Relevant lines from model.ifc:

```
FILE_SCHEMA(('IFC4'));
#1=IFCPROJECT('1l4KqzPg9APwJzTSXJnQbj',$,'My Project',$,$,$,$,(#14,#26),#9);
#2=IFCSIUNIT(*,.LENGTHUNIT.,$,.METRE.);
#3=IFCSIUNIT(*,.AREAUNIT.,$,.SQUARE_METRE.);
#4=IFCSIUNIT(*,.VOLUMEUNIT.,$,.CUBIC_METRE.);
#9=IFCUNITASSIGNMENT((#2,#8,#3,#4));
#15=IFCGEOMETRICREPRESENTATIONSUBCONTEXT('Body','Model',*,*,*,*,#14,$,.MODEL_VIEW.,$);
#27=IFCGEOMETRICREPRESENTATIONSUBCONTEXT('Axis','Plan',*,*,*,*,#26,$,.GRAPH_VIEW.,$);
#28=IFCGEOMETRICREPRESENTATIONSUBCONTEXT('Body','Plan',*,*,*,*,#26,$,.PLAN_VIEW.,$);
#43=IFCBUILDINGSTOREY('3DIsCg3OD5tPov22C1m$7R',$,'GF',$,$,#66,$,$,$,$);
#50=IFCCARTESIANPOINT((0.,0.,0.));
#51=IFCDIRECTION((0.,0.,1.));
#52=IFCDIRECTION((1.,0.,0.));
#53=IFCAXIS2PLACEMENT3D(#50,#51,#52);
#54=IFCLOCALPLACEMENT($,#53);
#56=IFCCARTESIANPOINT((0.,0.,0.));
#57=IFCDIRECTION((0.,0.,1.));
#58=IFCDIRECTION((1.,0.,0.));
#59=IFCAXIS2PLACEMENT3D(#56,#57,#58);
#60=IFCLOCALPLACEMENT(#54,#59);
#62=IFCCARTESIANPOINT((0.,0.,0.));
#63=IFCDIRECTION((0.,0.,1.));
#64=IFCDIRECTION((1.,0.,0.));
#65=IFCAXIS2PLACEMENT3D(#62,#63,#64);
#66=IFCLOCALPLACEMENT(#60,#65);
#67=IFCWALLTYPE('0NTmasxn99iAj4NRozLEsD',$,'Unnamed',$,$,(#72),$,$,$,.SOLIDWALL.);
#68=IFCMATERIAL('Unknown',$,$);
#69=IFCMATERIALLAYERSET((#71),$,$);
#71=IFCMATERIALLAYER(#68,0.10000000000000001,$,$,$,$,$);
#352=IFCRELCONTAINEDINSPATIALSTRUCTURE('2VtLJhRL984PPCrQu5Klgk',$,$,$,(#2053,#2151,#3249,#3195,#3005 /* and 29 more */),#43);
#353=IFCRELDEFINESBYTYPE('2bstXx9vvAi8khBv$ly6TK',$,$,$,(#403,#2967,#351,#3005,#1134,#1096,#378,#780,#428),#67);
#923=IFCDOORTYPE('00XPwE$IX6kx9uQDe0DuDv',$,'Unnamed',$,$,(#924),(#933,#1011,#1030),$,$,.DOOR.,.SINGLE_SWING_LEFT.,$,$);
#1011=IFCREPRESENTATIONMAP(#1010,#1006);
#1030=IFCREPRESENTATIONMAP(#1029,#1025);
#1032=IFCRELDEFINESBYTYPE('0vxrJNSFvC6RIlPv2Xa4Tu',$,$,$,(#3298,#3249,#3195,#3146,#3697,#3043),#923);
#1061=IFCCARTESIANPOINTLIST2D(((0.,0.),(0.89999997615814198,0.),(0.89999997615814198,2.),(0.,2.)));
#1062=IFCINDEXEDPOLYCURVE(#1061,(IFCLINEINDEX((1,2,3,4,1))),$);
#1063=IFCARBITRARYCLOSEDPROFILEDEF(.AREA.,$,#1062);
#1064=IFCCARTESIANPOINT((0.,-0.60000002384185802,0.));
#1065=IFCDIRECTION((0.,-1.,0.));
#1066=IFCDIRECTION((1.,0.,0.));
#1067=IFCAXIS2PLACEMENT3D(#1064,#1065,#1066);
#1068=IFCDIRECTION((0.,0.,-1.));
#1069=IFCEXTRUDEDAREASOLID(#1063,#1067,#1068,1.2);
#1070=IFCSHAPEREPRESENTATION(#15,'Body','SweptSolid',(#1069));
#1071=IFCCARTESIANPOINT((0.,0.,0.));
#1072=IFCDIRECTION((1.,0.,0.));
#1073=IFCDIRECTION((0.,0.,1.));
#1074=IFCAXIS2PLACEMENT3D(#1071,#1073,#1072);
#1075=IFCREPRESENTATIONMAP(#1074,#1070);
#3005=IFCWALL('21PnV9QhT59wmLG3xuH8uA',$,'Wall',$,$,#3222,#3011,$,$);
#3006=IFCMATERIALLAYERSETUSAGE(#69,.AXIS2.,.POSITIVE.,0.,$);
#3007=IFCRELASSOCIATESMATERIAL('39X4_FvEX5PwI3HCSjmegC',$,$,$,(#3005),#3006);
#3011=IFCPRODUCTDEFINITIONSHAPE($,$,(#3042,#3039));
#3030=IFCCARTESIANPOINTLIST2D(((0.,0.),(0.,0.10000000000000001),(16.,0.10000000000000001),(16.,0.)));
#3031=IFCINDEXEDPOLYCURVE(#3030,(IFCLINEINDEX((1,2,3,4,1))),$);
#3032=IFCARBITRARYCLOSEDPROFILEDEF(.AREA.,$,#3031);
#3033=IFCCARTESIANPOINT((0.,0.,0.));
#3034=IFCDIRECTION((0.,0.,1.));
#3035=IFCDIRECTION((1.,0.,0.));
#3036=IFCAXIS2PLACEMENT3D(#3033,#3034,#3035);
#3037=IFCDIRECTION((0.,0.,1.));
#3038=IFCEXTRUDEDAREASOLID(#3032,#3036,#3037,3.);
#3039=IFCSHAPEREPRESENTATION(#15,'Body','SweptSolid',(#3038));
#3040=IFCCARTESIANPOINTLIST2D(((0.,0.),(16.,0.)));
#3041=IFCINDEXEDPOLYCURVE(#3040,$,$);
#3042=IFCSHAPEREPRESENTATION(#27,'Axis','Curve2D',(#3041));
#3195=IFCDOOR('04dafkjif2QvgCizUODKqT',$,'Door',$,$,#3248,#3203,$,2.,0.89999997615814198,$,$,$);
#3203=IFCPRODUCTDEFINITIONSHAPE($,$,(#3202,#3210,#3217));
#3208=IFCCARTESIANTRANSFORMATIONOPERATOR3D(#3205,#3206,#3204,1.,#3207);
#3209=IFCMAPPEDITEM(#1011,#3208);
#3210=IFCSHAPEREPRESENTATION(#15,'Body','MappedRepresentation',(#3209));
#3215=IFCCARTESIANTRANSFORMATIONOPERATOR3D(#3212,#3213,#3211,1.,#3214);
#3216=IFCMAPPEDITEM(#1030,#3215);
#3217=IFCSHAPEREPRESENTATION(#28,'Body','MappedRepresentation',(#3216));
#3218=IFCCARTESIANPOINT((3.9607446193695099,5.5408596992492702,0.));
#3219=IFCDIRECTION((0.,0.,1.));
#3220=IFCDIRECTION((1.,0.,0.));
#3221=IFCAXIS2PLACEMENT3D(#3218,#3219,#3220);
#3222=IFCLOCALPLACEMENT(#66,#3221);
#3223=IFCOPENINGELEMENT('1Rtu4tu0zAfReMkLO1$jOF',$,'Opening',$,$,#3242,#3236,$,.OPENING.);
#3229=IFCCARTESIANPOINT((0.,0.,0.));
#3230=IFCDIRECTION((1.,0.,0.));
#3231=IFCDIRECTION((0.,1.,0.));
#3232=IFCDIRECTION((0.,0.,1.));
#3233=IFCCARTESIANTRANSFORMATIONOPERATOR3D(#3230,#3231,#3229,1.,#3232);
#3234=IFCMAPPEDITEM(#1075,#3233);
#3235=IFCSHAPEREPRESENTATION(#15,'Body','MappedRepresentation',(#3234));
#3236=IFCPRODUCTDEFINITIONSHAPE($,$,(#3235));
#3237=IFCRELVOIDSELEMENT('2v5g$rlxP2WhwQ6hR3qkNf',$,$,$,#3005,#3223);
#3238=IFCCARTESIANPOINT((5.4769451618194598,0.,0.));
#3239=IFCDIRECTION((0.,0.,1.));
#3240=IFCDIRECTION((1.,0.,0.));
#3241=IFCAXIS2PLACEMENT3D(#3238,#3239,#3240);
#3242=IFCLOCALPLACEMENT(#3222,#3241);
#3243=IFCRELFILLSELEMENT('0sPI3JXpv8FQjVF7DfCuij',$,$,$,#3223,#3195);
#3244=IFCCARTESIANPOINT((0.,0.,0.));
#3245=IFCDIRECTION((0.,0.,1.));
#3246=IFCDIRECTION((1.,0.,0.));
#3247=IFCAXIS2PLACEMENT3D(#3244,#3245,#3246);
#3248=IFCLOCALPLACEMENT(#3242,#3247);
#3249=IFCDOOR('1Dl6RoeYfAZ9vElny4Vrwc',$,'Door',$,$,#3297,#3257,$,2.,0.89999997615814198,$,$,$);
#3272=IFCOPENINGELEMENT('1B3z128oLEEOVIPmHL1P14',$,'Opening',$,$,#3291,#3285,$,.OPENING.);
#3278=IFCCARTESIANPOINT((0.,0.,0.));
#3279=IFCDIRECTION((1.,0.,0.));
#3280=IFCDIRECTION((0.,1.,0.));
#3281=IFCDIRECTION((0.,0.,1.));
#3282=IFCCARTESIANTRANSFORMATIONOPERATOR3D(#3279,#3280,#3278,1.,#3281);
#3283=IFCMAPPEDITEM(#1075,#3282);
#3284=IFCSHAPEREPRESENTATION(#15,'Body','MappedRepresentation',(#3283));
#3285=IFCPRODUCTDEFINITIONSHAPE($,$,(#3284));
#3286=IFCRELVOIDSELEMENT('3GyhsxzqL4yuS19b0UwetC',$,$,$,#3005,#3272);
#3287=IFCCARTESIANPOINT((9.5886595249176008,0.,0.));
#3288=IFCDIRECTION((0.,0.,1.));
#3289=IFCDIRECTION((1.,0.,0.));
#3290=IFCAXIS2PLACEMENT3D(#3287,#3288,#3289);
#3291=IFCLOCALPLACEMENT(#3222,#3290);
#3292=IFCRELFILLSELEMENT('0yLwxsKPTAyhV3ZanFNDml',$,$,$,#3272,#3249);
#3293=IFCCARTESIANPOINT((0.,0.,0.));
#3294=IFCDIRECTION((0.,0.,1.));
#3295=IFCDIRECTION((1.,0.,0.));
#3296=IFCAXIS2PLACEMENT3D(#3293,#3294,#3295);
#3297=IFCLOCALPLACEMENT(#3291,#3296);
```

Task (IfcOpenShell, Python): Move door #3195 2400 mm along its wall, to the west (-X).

```python
import ifcopenshell
import ifcopenshell.api.geometry
import ifcopenshell.util.placement
import ifcopenshell.util.unit

model = ifcopenshell.open("model.ifc")
unit_scale = ifcopenshell.util.unit.calculate_unit_scale(model)

door = model.by_guid("04dafkjif2QvgCizUODKqT")
opening = door.FillsVoids[0].RelatingOpeningElement
wall = opening.VoidsElements[0].RelatingBuildingElement

wall_matrix = ifcopenshell.util.placement.get_local_placement(wall.ObjectPlacement)
shift = wall_matrix[:3, 0] * -2.4 / unit_scale
before = ifcopenshell.util.placement.get_local_placement(door.ObjectPlacement)[:3, 3].copy()

# The door is placed relative to its opening, so it follows when the opening moves.
matrix = ifcopenshell.util.placement.get_local_placement(opening.ObjectPlacement)
matrix[:3, 3] += shift
ifcopenshell.api.geometry.edit_object_placement(
    model, product=opening, matrix=matrix, is_si=False, should_transform_children=True
)

after = ifcopenshell.util.placement.get_local_placement(door.ObjectPlacement)[:3, 3]
print("door moved by", (after - before).round(3) + 0.0)

model.write("model_v2.ifc")
```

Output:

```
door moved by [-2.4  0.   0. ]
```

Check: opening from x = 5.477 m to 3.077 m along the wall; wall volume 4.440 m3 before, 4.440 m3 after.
